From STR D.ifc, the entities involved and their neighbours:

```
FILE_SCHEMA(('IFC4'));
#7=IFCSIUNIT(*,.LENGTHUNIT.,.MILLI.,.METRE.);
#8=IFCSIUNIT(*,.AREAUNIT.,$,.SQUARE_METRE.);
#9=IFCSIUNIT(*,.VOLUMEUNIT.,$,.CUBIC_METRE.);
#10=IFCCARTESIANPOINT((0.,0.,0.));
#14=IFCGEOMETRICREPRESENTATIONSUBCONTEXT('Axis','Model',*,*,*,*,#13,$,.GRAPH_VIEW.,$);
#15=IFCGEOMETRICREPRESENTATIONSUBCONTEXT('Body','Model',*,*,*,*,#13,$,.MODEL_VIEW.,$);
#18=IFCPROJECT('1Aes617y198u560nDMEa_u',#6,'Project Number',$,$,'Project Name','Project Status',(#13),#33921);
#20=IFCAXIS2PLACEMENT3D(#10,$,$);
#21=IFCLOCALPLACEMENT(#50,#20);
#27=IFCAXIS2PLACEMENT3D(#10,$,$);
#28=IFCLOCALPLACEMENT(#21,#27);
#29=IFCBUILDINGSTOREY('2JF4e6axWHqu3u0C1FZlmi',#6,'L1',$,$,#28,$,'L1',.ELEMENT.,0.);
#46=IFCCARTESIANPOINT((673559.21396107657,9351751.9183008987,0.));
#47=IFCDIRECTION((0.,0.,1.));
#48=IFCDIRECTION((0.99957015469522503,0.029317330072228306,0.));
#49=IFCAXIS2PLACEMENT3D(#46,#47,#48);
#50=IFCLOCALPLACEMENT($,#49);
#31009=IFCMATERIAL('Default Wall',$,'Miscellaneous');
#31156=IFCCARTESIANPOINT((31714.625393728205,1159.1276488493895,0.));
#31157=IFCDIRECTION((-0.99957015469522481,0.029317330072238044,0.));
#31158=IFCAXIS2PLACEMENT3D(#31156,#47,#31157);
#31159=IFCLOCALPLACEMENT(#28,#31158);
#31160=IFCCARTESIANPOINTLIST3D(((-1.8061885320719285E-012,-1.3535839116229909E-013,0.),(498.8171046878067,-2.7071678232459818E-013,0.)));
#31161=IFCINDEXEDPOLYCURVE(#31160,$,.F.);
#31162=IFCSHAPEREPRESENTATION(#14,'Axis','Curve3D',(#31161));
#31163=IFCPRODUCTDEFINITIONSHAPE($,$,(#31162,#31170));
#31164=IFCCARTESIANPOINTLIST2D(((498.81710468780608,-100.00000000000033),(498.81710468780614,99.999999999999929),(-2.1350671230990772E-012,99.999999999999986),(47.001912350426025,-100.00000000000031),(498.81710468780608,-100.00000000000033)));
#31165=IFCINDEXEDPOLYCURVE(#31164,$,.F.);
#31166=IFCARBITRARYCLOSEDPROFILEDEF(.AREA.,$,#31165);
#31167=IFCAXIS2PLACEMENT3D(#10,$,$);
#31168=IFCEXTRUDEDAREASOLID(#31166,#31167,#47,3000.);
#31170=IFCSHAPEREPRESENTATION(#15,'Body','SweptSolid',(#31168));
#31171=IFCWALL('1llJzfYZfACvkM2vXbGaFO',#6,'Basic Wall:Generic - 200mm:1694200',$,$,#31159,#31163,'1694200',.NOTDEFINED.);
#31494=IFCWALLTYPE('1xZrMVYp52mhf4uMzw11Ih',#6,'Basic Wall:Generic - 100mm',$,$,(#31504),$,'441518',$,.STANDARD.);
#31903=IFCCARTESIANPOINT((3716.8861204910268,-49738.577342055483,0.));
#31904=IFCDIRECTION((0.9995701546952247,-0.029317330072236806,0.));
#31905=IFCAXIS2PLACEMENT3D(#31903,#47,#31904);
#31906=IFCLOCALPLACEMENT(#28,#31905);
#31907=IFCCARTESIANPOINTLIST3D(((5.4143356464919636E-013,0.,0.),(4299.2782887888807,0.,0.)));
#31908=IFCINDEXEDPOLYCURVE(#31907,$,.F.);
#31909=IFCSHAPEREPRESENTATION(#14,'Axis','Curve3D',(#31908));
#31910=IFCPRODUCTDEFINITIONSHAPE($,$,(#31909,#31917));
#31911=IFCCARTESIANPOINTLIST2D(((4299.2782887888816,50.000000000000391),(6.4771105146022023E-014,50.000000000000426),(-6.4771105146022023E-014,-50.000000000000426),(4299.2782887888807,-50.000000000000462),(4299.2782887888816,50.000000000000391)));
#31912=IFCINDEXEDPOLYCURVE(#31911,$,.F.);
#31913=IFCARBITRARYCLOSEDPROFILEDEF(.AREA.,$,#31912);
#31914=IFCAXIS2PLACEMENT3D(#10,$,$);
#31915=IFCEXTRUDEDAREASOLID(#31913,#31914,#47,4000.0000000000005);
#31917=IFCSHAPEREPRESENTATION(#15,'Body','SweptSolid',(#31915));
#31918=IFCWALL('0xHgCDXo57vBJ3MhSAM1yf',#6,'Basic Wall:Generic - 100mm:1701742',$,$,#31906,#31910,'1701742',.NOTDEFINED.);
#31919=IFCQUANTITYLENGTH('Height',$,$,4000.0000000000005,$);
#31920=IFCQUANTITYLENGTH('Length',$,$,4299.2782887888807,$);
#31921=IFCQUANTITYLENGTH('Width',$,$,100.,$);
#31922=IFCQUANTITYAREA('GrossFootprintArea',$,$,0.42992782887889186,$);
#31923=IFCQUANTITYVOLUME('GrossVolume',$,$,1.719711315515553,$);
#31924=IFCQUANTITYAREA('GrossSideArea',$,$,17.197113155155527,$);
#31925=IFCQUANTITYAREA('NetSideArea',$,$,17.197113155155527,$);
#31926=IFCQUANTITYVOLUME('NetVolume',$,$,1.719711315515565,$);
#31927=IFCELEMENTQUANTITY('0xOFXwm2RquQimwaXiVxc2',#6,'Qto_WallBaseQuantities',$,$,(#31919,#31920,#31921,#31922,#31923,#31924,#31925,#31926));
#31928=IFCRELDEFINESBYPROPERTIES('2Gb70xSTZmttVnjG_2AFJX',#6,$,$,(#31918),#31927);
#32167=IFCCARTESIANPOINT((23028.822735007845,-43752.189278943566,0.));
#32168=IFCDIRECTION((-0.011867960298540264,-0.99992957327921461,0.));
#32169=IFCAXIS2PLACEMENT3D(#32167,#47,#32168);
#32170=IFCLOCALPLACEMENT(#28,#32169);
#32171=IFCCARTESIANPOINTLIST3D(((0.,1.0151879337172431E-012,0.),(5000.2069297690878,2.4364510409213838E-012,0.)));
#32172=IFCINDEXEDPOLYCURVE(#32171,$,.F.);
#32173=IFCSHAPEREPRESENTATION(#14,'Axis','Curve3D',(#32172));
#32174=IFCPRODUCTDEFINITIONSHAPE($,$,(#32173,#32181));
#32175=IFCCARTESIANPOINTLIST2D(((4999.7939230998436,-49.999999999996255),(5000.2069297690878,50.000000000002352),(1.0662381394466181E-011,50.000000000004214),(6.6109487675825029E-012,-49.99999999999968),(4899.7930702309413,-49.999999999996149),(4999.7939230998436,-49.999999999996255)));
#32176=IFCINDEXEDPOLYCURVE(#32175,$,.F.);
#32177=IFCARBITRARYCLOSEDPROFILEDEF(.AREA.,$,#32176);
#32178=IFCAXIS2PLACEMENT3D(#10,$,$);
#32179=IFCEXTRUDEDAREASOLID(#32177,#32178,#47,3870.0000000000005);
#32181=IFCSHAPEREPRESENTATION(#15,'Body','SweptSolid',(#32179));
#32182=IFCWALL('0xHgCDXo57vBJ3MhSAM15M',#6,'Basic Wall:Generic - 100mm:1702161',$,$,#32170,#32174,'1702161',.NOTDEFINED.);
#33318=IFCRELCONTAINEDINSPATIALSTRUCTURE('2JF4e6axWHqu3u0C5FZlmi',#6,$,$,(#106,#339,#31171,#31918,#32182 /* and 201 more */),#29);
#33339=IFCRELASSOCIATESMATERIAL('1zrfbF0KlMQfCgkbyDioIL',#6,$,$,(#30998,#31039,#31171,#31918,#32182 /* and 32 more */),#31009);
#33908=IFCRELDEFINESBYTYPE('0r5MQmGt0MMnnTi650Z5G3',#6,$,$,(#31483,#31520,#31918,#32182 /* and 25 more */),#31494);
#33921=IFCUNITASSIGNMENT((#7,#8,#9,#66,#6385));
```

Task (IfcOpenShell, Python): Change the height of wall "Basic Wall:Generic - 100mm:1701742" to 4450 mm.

```python
import ifcopenshell
import ifcopenshell.api.pset
import ifcopenshell.geom
import ifcopenshell.util.element
import ifcopenshell.util.representation
import ifcopenshell.util.shape
import ifcopenshell.util.unit

model = ifcopenshell.open("STR D.ifc")
unit_scale = ifcopenshell.util.unit.calculate_unit_scale(model)
area_scale = ifcopenshell.util.unit.calculate_unit_scale(model, "AREAUNIT")
volume_scale = ifcopenshell.util.unit.calculate_unit_scale(model, "VOLUMEUNIT")
settings = ifcopenshell.geom.settings()


def volume(element):
    """Net volume in cubic metres, openings subtracted."""
    shape = ifcopenshell.geom.create_shape(settings, element)
    return ifcopenshell.util.shape.get_volume(shape.geometry)


wall = model.by_guid("0xHgCDXo57vBJ3MhSAM1yf")
before = volume(wall)

body = ifcopenshell.util.representation.get_representation(wall, "Model", "Body")
solid = body.Items[0]
old_height = solid.Depth
solid.Depth = 4.45 / unit_scale
after = volume(wall)
thickness = 0.1  # wall thickness in metres

# Update the stored height, areas and volumes.
qto = model.by_id(ifcopenshell.util.element.get_pset(wall, "Qto_WallBaseQuantities", should_inherit=False)["id"])
ifcopenshell.api.pset.edit_qto(model, qto=qto, properties={
    "Height": solid.Depth,
    "GrossVolume": ifcopenshell.util.element.get_pset(wall, "Qto_WallBaseQuantities", "GrossVolume") * solid.Depth / old_height,
    "GrossSideArea": ifcopenshell.util.element.get_pset(wall, "Qto_WallBaseQuantities", "GrossSideArea") * solid.Depth / old_height,
    "NetSideArea": after / thickness / area_scale,
    "NetVolume": after / volume_scale,
})

print(f"height {old_height:g} -> {solid.Depth:g}, volume {before:.3f} -> {after:.3f} m3")

model.write("STR D_updated.ifc")
```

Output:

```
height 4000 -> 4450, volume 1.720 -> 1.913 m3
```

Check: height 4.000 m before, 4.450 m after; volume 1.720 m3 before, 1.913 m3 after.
